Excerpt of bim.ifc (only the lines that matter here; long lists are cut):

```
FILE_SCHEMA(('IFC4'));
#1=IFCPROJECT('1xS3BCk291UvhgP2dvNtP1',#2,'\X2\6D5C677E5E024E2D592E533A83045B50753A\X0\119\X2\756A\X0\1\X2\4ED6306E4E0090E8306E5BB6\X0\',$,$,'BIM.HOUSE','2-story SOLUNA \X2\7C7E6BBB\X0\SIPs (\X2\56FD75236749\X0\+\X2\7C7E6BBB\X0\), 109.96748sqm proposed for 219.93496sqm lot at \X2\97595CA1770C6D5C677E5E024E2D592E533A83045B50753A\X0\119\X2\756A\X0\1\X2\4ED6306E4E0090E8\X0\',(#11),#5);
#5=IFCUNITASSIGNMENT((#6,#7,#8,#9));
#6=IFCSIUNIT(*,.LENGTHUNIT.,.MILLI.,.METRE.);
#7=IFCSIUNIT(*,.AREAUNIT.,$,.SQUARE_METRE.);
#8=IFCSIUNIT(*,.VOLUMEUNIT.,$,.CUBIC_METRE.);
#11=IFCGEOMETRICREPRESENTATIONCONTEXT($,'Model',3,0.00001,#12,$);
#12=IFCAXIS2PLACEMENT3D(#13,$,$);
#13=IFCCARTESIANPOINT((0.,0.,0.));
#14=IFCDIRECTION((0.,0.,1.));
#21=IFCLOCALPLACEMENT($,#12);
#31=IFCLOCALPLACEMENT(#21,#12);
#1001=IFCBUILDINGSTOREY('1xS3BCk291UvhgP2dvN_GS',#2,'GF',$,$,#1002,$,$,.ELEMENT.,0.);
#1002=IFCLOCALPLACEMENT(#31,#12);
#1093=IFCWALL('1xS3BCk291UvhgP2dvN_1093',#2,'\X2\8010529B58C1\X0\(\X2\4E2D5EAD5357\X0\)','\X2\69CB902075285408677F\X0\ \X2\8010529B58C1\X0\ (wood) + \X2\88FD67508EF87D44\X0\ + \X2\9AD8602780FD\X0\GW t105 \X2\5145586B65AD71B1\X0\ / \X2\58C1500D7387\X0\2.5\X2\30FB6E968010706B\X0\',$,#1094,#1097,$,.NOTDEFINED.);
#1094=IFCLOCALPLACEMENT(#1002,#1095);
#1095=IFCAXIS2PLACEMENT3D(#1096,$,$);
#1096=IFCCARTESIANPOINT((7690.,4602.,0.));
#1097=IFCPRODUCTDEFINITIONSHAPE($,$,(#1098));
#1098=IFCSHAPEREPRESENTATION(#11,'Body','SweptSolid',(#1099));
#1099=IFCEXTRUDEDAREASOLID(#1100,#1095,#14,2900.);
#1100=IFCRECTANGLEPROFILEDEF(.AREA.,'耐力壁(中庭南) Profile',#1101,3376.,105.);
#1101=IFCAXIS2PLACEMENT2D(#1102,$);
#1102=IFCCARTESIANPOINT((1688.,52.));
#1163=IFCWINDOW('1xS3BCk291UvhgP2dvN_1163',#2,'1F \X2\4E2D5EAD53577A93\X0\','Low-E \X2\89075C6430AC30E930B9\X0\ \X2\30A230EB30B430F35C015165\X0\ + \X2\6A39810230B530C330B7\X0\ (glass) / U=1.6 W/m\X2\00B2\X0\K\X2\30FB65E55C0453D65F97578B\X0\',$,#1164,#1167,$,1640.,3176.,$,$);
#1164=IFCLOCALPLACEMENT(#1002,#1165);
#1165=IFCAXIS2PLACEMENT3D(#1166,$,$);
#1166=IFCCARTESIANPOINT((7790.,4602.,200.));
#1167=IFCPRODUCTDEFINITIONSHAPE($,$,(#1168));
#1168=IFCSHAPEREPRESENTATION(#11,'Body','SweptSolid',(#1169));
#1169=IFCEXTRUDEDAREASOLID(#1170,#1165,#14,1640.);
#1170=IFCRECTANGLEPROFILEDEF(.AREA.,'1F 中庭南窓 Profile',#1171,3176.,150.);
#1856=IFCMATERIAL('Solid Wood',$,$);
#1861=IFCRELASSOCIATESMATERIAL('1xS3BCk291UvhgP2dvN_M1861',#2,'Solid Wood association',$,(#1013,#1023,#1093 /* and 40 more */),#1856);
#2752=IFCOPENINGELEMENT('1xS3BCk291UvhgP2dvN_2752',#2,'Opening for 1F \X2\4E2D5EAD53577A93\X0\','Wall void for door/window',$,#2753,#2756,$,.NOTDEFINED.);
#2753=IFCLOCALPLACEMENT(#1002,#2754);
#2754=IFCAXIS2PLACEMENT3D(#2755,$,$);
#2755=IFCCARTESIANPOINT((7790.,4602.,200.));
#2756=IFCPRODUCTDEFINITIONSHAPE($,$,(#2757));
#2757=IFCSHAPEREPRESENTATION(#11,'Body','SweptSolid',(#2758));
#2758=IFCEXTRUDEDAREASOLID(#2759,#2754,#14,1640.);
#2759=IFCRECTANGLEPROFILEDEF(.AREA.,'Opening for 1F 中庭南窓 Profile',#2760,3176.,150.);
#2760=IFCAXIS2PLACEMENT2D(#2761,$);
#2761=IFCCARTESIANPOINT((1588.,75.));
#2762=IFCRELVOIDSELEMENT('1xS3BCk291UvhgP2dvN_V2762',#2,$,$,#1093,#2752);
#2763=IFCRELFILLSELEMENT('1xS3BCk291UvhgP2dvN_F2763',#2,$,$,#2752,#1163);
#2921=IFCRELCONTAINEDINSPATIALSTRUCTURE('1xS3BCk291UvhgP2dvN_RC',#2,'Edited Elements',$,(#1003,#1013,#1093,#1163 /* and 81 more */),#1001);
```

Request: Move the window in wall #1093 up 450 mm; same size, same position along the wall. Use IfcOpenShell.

```python
import numpy as np
import ifcopenshell
import ifcopenshell.api.geometry
import ifcopenshell.util.placement
import ifcopenshell.util.unit

model = ifcopenshell.open("bim.ifc")
unit_scale = ifcopenshell.util.unit.calculate_unit_scale(model)

window = model.by_guid("1xS3BCk291UvhgP2dvN_1163")
opening = window.FillsVoids[0].RelatingOpeningElement
dz = 0.45 / unit_scale

shift = np.array([0.0, 0.0, dz])
# The window is not placed relative to its opening, so move both.
for product in (opening, window):
    matrix = ifcopenshell.util.placement.get_local_placement(product.ObjectPlacement)
    matrix[:3, 3] += shift
    ifcopenshell.api.geometry.edit_object_placement(model, product=product, matrix=matrix, is_si=False)

print(f"moved by {dz * unit_scale:+.3f} m")

model.write("bim_rev.ifc")
```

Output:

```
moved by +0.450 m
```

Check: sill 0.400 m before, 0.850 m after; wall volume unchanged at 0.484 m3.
